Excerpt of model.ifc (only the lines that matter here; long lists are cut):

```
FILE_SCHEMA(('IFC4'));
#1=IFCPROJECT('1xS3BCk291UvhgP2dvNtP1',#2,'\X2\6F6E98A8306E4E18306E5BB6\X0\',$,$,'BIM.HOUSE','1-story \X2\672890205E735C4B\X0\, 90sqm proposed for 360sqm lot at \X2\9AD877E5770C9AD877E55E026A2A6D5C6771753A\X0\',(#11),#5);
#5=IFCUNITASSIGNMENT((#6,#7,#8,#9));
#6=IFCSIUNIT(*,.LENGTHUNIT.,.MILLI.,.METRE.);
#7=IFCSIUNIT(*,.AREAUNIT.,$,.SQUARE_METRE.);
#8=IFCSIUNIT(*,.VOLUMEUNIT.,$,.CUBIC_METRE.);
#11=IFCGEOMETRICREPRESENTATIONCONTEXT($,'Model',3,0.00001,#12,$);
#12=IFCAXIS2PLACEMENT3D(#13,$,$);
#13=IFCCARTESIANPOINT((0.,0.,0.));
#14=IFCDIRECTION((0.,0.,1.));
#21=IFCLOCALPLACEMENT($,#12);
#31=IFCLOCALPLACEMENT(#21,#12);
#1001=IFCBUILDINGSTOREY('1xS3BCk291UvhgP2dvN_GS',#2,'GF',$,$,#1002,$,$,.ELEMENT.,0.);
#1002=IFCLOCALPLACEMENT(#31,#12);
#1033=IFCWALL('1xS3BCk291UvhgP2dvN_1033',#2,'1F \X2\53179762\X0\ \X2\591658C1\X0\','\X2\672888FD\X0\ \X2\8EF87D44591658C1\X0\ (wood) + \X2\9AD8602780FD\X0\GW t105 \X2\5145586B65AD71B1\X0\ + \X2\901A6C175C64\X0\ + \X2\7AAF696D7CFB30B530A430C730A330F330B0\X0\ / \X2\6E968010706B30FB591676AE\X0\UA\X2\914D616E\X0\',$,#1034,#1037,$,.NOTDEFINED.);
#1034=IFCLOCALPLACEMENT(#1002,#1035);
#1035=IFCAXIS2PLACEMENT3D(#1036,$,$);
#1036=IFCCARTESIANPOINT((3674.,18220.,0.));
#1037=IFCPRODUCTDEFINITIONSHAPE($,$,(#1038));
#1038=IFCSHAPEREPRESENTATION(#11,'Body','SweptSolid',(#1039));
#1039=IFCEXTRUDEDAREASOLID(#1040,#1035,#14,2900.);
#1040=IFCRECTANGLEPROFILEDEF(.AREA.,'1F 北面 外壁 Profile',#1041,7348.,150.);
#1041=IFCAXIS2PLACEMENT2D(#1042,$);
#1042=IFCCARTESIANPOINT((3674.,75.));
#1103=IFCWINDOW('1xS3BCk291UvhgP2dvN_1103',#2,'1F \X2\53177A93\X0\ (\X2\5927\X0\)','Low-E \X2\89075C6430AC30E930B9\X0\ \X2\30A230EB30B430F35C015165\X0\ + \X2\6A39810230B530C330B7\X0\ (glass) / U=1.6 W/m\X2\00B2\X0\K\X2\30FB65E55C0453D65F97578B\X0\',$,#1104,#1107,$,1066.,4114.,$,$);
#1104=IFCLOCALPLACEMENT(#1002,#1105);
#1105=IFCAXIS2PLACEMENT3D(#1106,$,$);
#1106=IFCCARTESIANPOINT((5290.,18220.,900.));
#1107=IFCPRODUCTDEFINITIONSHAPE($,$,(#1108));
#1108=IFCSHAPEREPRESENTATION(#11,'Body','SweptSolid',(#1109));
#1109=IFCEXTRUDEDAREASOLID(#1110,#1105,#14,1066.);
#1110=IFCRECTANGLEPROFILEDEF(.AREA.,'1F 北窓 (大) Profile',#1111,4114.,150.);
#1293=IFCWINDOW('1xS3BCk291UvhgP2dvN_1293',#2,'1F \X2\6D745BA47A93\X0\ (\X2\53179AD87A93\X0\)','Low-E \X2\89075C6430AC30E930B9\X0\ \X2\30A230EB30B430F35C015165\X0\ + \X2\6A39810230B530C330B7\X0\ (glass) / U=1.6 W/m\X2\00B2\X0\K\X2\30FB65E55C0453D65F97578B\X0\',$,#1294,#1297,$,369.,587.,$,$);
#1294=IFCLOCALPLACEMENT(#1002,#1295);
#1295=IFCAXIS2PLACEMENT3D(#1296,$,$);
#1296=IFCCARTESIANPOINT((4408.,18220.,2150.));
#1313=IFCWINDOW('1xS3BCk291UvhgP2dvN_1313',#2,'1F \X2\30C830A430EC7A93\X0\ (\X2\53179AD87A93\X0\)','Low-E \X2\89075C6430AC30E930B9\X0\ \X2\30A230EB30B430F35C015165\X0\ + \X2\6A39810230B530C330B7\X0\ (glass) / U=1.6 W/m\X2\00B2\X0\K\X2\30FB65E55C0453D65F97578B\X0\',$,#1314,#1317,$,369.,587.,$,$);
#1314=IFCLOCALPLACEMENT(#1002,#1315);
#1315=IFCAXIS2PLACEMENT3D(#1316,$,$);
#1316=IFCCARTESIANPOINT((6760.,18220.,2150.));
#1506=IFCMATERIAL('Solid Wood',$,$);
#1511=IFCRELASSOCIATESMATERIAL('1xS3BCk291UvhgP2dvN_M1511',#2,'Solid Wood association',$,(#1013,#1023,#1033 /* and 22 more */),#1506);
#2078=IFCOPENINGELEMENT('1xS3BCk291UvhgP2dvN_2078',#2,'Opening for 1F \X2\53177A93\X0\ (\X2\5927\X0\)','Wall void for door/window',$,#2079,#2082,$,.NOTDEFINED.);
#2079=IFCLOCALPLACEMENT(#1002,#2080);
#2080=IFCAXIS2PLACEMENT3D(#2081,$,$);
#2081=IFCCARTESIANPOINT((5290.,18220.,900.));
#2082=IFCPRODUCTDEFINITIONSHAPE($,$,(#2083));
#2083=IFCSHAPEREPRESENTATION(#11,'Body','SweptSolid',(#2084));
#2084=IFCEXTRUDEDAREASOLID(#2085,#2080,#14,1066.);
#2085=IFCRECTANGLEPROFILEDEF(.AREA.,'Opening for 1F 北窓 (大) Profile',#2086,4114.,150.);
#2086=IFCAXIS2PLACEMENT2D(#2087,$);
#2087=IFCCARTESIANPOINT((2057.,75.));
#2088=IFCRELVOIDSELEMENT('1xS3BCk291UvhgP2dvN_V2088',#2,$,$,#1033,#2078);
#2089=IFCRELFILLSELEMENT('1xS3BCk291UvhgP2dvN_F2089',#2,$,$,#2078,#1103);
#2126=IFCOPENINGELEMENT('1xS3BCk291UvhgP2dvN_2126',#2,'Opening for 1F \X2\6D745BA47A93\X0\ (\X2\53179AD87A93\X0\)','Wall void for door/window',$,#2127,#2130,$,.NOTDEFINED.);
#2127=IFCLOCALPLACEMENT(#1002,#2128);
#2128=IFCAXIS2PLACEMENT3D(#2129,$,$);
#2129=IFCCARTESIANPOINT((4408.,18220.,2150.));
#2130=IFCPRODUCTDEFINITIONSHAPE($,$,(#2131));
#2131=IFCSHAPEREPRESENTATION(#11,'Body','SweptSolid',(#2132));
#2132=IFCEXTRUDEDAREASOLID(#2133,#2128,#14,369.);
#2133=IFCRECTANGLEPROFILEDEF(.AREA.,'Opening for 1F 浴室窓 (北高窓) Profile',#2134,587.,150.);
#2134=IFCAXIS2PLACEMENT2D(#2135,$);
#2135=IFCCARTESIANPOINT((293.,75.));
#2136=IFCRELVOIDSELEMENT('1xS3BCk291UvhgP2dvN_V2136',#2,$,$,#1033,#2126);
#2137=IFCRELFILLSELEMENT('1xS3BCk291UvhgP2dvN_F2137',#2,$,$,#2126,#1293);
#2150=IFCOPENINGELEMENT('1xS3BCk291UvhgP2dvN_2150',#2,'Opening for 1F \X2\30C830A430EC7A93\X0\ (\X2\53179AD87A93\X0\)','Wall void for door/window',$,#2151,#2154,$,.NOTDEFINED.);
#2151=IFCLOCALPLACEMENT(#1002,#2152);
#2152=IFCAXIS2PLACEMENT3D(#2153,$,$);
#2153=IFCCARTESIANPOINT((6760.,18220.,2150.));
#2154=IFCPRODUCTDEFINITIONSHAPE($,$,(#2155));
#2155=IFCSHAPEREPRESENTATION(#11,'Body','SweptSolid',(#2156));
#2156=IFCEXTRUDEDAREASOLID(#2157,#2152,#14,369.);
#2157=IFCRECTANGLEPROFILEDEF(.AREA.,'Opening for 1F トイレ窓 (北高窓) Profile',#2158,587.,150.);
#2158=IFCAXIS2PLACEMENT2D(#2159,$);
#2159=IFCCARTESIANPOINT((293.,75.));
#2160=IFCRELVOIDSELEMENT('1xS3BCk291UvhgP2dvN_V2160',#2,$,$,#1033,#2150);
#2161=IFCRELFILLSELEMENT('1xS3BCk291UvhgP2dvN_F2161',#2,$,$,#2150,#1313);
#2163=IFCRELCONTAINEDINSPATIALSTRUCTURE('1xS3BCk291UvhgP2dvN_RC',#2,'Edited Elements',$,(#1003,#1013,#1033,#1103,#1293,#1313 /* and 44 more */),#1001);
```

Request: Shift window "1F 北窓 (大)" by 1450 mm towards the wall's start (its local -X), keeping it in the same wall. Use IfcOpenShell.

```python
import ifcopenshell
import ifcopenshell.api.geometry
import ifcopenshell.util.placement
import ifcopenshell.util.unit

model = ifcopenshell.open("model.ifc")
unit_scale = ifcopenshell.util.unit.calculate_unit_scale(model)

window = model.by_guid("1xS3BCk291UvhgP2dvN_1103")
opening = window.FillsVoids[0].RelatingOpeningElement
wall = opening.VoidsElements[0].RelatingBuildingElement

wall_matrix = ifcopenshell.util.placement.get_local_placement(wall.ObjectPlacement)
shift = wall_matrix[:3, 0] * -1.45 / unit_scale
before = ifcopenshell.util.placement.get_local_placement(window.ObjectPlacement)[:3, 3].copy()

# The window is not placed relative to its opening, so move both.
for product in (opening, window):
    matrix = ifcopenshell.util.placement.get_local_placement(product.ObjectPlacement)
    matrix[:3, 3] += shift
    ifcopenshell.api.geometry.edit_object_placement(model, product=product, matrix=matrix, is_si=False)

after = ifcopenshell.util.placement.get_local_placement(window.ObjectPlacement)[:3, 3]
print("window moved by", (after - before).round(3) + 0.0)

model.write("model_edited.ifc")
```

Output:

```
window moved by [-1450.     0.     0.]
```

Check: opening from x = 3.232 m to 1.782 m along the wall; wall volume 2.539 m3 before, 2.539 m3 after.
